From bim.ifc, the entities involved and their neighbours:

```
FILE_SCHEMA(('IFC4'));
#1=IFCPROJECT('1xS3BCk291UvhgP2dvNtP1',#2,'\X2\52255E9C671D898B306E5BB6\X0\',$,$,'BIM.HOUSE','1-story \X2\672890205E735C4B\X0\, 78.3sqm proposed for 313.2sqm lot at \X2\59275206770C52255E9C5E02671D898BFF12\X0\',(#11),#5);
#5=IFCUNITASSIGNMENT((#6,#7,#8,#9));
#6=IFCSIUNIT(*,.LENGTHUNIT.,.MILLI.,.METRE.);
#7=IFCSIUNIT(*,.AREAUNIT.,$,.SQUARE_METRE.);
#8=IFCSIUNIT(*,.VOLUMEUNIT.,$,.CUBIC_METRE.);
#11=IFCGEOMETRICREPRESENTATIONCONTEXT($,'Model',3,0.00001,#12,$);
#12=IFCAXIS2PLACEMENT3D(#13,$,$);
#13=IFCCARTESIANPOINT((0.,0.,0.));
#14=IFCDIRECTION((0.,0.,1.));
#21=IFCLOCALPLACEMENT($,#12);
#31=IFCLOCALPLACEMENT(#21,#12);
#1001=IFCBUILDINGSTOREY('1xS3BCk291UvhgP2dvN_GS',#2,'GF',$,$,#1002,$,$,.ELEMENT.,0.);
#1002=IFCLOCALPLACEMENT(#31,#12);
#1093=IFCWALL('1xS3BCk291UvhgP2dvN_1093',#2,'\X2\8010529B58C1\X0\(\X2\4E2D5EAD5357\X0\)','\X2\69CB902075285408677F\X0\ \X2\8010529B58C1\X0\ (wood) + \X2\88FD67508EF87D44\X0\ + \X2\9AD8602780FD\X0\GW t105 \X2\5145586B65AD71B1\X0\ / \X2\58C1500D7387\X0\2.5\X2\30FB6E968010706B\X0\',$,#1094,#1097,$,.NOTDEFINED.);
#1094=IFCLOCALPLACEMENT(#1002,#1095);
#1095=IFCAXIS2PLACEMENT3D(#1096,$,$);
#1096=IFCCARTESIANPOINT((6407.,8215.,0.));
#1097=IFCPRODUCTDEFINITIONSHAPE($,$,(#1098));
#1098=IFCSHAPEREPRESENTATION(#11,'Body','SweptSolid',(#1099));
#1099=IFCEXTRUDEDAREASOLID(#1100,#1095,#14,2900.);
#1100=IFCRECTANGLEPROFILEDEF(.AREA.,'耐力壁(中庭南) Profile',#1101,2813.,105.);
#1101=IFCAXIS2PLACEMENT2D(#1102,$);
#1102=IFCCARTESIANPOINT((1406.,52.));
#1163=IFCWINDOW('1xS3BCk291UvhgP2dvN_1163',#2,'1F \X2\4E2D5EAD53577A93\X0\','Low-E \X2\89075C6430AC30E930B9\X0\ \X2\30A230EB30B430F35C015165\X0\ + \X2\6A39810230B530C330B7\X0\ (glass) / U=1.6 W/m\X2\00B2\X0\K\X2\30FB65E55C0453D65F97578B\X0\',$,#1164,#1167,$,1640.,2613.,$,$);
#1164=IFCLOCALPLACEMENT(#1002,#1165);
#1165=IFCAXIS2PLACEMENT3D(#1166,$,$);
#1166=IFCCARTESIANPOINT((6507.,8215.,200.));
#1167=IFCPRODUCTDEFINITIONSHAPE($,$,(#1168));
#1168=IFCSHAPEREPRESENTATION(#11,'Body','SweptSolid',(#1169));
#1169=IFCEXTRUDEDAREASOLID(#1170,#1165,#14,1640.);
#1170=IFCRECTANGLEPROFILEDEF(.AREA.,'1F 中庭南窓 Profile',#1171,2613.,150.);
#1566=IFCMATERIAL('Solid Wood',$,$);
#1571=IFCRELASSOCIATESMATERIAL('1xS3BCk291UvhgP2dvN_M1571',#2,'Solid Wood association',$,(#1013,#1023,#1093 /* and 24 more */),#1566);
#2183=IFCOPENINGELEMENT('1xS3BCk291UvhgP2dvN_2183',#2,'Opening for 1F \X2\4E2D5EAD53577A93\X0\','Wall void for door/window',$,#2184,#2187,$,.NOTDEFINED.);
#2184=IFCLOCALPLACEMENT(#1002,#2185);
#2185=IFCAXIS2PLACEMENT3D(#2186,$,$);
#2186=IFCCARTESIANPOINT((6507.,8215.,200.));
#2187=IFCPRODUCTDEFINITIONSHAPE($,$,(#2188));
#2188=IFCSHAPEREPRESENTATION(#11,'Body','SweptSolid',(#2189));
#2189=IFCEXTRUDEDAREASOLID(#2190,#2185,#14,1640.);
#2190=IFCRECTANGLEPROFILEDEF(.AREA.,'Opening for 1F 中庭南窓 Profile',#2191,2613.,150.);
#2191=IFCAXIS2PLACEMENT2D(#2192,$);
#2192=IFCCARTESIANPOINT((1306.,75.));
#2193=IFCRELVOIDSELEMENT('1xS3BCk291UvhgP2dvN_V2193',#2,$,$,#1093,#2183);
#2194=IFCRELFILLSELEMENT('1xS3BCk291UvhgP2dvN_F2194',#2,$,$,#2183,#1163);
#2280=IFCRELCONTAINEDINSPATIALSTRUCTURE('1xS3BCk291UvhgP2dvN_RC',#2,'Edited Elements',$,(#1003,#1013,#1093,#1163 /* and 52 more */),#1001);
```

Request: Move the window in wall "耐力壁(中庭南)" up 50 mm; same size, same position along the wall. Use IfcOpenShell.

```python
import numpy as np
import ifcopenshell
import ifcopenshell.api.geometry
import ifcopenshell.util.placement
import ifcopenshell.util.unit

model = ifcopenshell.open("bim.ifc")
unit_scale = ifcopenshell.util.unit.calculate_unit_scale(model)

window = model.by_guid("1xS3BCk291UvhgP2dvN_1163")
opening = window.FillsVoids[0].RelatingOpeningElement
dz = 0.05 / unit_scale

shift = np.array([0.0, 0.0, dz])
# The window is not placed relative to its opening, so move both.
for product in (opening, window):
    matrix = ifcopenshell.util.placement.get_local_placement(product.ObjectPlacement)
    matrix[:3, 3] += shift
    ifcopenshell.api.geometry.edit_object_placement(model, product=product, matrix=matrix, is_si=False)

print(f"moved by {dz * unit_scale:+.3f} m")

model.write("bim_updated.ifc")
```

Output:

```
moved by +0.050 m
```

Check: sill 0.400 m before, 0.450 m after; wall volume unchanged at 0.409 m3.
